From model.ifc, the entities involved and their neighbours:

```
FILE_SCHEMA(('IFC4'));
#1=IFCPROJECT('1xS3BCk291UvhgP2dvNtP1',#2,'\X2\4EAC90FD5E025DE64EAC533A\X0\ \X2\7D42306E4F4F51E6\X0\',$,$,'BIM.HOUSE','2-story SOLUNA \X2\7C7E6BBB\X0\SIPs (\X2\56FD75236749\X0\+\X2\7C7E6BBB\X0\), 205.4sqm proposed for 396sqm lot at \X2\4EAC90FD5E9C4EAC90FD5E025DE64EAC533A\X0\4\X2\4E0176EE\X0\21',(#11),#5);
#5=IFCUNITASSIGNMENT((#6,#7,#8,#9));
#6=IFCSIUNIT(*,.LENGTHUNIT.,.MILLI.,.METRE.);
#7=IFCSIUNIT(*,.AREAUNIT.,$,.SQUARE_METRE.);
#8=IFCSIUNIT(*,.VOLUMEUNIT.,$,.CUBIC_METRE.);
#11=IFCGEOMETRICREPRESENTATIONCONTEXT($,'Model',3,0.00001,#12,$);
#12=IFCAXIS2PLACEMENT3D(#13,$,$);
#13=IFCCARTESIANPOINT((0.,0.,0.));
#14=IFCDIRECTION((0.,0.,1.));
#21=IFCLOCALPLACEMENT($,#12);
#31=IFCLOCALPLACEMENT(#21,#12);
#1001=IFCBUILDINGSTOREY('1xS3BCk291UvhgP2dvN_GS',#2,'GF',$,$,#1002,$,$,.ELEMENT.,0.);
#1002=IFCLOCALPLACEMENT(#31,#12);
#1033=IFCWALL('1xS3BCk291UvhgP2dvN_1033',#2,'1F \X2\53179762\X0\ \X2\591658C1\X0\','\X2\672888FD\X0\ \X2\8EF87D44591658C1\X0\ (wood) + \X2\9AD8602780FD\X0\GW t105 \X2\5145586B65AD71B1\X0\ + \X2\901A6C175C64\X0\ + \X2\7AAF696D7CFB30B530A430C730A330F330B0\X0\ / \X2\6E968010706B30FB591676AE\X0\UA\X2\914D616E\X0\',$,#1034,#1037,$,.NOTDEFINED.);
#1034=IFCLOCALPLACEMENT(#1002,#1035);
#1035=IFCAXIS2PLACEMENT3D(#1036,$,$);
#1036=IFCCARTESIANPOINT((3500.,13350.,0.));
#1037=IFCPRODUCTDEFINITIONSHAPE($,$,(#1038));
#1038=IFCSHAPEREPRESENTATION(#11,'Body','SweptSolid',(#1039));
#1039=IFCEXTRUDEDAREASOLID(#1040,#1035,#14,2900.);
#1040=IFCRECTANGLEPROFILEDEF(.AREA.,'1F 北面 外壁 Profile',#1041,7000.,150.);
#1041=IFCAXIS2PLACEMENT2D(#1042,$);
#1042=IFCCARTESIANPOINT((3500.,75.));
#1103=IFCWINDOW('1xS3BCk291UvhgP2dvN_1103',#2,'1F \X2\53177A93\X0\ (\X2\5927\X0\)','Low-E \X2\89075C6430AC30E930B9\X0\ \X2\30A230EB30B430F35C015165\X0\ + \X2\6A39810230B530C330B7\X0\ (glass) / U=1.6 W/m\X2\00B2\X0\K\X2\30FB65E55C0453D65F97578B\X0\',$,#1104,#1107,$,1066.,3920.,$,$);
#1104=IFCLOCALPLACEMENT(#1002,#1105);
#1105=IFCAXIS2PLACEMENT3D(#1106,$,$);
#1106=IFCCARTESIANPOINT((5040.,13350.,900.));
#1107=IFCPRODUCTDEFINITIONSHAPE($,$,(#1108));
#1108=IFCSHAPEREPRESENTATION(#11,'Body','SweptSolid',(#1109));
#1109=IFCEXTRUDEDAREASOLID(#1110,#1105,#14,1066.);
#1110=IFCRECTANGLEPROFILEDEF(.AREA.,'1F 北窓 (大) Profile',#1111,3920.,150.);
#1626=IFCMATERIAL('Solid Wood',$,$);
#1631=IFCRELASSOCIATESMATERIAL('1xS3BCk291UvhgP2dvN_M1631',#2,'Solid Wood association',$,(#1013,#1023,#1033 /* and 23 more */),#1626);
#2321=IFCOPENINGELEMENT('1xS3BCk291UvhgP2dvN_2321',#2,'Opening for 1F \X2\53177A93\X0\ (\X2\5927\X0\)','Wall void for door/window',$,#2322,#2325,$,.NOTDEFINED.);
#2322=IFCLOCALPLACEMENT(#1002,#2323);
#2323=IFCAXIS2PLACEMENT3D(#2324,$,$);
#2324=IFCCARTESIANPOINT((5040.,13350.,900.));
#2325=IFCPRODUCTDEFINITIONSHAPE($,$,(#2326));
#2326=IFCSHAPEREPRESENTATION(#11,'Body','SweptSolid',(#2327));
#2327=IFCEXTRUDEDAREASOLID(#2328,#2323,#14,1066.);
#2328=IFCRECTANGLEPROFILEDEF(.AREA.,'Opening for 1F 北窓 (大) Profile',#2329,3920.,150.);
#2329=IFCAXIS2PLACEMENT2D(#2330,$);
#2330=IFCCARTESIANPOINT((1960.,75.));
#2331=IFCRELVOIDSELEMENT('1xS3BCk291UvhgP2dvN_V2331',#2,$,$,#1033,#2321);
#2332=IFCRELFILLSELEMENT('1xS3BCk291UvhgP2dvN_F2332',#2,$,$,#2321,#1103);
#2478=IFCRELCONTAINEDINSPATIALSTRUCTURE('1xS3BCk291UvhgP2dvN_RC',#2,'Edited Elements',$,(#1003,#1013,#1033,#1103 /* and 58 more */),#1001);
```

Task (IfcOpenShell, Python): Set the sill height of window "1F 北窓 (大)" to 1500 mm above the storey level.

```python
import numpy as np
import ifcopenshell
import ifcopenshell.api.geometry
import ifcopenshell.geom
import ifcopenshell.util.element
import ifcopenshell.util.placement
import ifcopenshell.util.shape
import ifcopenshell.util.unit

model = ifcopenshell.open("model.ifc")
unit_scale = ifcopenshell.util.unit.calculate_unit_scale(model)

window = model.by_guid("1xS3BCk291UvhgP2dvN_1103")
opening = window.FillsVoids[0].RelatingOpeningElement
storey = ifcopenshell.util.element.get_container(window, ifc_class="IfcBuildingStorey")
level = ifcopenshell.util.placement.get_local_placement(storey.ObjectPlacement)[2, 3]

# The opening's origin need not be at the sill, so measure its lowest point.
shape = ifcopenshell.geom.create_shape(ifcopenshell.geom.settings(), opening)
bottom = ifcopenshell.util.shape.get_shape_bottom_elevation(shape, shape.geometry) / unit_scale
dz = level + 1.5 / unit_scale - bottom

shift = np.array([0.0, 0.0, dz])
# The window is not placed relative to its opening, so move both.
for product in (opening, window):
    matrix = ifcopenshell.util.placement.get_local_placement(product.ObjectPlacement)
    matrix[:3, 3] += shift
    ifcopenshell.api.geometry.edit_object_placement(model, product=product, matrix=matrix, is_si=False)

print(f"moved by {dz * unit_scale:+.3f} m")

model.write("model_v2.ifc")
```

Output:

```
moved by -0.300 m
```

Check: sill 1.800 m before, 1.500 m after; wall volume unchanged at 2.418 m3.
